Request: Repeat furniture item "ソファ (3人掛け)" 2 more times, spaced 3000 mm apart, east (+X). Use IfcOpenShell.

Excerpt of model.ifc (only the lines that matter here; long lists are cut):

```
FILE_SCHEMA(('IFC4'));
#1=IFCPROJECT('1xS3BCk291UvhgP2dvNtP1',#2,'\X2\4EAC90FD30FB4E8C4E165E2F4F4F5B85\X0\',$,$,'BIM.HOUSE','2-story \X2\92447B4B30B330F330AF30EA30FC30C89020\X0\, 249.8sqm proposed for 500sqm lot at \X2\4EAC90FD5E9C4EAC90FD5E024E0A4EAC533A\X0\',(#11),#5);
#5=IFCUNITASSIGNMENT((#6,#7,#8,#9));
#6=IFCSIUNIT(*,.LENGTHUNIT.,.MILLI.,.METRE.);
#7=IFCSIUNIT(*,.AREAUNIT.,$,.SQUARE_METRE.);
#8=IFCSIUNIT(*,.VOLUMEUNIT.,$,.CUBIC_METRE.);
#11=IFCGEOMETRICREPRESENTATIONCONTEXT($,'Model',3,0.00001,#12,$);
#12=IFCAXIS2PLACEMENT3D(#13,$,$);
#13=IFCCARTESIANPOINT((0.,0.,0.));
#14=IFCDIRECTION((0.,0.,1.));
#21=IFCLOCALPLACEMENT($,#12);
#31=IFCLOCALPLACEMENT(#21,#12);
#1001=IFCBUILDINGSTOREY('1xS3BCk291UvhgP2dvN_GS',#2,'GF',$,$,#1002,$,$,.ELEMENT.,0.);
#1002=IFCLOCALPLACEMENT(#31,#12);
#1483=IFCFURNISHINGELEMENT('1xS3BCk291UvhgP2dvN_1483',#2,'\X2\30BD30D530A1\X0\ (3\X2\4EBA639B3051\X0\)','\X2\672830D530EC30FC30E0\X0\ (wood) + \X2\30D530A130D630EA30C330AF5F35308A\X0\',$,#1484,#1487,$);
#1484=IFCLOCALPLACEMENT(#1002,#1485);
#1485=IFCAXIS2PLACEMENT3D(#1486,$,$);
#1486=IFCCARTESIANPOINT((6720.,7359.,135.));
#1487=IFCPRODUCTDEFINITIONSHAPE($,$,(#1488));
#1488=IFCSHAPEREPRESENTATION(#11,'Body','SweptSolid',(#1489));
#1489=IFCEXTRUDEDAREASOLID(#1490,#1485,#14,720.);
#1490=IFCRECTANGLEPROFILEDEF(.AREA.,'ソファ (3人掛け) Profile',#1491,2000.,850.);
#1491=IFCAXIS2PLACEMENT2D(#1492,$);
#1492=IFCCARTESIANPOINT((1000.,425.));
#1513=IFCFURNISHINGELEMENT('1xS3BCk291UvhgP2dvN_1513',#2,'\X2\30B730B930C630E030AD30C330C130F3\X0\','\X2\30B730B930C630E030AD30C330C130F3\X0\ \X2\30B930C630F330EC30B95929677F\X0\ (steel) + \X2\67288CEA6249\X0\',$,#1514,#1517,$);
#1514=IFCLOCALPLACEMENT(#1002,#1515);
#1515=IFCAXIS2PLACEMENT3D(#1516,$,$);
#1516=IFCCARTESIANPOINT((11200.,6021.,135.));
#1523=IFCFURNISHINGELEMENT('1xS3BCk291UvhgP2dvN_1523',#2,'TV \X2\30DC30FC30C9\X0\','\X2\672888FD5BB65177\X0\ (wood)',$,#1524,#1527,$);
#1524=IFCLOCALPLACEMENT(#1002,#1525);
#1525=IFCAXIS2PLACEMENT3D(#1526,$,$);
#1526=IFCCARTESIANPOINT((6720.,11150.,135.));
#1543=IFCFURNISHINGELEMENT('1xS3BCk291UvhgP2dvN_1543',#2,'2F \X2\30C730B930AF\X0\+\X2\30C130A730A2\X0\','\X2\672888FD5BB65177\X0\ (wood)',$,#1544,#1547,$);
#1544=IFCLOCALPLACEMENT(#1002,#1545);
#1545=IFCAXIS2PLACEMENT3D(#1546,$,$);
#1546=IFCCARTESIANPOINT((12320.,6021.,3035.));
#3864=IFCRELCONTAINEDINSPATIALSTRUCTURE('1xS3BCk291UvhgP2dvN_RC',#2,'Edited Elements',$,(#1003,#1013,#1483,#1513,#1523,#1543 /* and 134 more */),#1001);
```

```python
import numpy as np
import ifcopenshell
import ifcopenshell.api.geometry
import ifcopenshell.api.root
import ifcopenshell.util.element
import ifcopenshell.util.placement

model = ifcopenshell.open("model.ifc")


def reuse_history(source, copy):
    """copy_class also copies each property set's owner history, people and application; keep the originals."""
    for rel in copy.IsDefinedBy:
        if rel.is_a("IfcRelDefinesByProperties") and (history := rel.RelatingPropertyDefinition.OwnerHistory):
            rel.RelatingPropertyDefinition.OwnerHistory = source.OwnerHistory
            ifcopenshell.util.element.remove_deep2(model, history)


source = model.by_guid("1xS3BCk291UvhgP2dvN_1483")
base = ifcopenshell.util.placement.get_local_placement(source.ObjectPlacement)
step = np.array([1.0, 0.0, 0.0]) * 3000.0

for i in range(1, 3):
    copy = ifcopenshell.api.root.copy_class(model, product=source)
    copy.Representation = ifcopenshell.util.element.copy_deep(
        model, source.Representation, exclude=["IfcGeometricRepresentationContext", "IfcRepresentationMap"]
    )
    reuse_history(source, copy)
    matrix = base.copy()
    matrix[:3, 3] += i * step
    print("added at", matrix[:3, 3].round(3) + 0.0)
    ifcopenshell.api.geometry.edit_object_placement(model, product=copy, matrix=matrix, is_si=False)

model.write("model_edited.ifc")
```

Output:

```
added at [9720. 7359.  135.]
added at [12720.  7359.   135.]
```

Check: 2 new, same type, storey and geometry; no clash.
